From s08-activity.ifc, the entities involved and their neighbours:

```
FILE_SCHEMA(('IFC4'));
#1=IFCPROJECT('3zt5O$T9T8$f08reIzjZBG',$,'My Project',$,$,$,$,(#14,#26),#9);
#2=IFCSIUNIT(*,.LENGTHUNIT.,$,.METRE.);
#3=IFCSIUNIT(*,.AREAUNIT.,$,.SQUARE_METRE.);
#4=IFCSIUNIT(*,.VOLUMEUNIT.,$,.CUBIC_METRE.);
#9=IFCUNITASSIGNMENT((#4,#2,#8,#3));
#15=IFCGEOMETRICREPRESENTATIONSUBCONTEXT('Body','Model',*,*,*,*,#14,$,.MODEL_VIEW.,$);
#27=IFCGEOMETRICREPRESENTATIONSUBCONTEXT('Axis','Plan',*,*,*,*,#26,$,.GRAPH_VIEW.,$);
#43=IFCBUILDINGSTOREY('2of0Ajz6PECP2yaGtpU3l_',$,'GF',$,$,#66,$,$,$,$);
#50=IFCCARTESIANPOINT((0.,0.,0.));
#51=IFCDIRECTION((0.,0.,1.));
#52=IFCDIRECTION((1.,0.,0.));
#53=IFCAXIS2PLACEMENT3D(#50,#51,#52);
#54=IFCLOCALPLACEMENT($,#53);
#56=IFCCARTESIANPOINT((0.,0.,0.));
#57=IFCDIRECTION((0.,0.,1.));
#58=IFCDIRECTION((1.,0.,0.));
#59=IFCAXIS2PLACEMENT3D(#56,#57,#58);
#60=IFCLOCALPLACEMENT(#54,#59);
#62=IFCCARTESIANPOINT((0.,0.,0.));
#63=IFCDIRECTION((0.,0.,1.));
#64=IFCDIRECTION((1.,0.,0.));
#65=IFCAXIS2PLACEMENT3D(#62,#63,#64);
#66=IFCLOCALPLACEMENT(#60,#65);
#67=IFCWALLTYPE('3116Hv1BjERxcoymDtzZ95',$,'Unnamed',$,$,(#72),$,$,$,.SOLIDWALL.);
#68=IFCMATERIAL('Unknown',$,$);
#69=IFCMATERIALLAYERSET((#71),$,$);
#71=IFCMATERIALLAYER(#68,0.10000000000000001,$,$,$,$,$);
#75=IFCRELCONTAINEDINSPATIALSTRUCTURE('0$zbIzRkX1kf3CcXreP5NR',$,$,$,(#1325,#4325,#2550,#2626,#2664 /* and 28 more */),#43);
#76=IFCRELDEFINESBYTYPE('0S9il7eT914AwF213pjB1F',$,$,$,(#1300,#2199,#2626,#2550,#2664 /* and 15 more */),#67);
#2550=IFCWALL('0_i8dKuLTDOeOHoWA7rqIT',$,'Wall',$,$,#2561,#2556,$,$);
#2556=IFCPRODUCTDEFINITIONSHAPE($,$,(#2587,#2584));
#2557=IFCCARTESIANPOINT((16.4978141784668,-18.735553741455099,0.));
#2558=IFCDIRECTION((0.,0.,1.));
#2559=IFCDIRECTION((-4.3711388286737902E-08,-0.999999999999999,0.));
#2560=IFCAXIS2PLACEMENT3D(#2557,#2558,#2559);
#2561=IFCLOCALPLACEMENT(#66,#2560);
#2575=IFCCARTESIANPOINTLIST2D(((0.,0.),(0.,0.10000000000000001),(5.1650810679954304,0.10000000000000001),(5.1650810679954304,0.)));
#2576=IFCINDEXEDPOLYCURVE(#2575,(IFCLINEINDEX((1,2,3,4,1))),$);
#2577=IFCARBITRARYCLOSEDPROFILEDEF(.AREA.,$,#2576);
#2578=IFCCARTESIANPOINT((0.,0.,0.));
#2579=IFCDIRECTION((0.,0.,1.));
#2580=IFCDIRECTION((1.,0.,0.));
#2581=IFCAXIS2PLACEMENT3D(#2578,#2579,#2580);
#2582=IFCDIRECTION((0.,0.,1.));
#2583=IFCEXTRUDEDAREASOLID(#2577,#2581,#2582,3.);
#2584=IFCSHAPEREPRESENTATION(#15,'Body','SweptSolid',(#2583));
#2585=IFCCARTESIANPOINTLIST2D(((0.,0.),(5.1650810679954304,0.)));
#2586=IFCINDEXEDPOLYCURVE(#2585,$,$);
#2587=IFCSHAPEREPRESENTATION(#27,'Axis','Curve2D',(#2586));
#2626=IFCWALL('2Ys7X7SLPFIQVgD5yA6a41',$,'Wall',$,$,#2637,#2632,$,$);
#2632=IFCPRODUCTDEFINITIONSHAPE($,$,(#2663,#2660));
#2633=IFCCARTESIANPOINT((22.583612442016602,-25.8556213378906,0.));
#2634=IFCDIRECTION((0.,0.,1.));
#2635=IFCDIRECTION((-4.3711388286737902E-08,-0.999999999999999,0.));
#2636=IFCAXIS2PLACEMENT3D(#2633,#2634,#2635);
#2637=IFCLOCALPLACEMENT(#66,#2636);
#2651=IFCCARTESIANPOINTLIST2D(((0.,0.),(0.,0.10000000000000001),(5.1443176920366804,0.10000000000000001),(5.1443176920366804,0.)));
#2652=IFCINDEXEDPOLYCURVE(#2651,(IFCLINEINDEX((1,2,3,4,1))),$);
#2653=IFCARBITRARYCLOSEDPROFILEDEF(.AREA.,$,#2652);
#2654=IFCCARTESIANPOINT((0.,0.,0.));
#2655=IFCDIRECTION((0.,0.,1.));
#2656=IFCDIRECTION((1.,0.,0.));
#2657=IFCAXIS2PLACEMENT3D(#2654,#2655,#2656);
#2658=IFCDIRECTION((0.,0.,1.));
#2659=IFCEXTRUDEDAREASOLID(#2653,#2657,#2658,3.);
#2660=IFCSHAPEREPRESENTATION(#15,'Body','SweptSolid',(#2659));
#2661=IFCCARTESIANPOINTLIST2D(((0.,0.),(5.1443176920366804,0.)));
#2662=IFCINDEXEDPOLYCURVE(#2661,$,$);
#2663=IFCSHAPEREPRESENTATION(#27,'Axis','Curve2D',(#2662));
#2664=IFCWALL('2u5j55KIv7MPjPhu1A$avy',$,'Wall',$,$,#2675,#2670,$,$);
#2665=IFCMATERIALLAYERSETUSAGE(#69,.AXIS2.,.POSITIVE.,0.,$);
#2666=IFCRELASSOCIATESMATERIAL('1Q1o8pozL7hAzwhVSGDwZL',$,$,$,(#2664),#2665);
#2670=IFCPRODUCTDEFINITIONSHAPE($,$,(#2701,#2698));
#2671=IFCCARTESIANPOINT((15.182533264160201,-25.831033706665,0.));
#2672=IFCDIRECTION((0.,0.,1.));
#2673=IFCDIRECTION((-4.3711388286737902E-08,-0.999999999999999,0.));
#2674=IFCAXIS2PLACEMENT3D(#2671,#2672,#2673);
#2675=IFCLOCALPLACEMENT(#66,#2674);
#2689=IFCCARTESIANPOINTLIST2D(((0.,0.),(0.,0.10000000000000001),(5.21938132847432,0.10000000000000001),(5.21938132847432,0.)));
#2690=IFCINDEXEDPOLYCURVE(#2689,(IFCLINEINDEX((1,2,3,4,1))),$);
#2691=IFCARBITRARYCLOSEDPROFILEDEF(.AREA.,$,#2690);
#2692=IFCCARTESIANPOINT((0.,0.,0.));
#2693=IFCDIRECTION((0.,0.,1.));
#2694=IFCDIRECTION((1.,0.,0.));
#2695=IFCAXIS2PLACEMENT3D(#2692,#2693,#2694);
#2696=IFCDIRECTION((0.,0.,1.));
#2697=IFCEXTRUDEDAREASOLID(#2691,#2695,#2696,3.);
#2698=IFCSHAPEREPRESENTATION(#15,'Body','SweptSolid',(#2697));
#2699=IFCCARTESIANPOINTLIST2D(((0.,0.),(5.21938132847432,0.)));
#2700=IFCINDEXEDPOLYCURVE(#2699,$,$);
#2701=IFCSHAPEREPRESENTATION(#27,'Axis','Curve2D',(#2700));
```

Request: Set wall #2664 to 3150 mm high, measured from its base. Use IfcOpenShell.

```python
import ifcopenshell
import ifcopenshell.geom
import ifcopenshell.util.representation
import ifcopenshell.util.shape
import ifcopenshell.util.unit

model = ifcopenshell.open("s08-activity.ifc")
unit_scale = ifcopenshell.util.unit.calculate_unit_scale(model)
settings = ifcopenshell.geom.settings()


def volume(element):
    """Net volume in cubic metres, openings subtracted."""
    shape = ifcopenshell.geom.create_shape(settings, element)
    return ifcopenshell.util.shape.get_volume(shape.geometry)


wall = model.by_guid("2u5j55KIv7MPjPhu1A$avy")
before = volume(wall)

body = ifcopenshell.util.representation.get_representation(wall, "Model", "Body")
solid = body.Items[0]
old_height = solid.Depth
solid.Depth = 3.15 / unit_scale
after = volume(wall)

print(f"height {old_height:g} -> {solid.Depth:g}, volume {before:.3f} -> {after:.3f} m3")

model.write("s08-activity_rev.ifc")
```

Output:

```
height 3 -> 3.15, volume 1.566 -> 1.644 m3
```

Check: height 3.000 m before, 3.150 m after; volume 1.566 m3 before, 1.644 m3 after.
